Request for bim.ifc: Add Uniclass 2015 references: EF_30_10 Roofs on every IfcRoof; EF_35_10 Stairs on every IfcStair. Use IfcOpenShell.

First a look at what the model holds.

```python
import ifcopenshell

model = ifcopenshell.open("bim.ifc")
print(model.schema)
print("classifications:", [c.Name for c in model.by_type("IfcClassification")])
for ifc_class in ("IfcDoor", "IfcRoof", "IfcStair", "IfcWall", "IfcWindow"):
    print(ifc_class, len(model.by_type(ifc_class)))
```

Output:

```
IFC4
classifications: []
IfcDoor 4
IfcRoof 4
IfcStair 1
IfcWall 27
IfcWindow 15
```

```python
import ifcopenshell
import ifcopenshell.api.classification

model = ifcopenshell.open("bim.ifc")

system = ifcopenshell.api.classification.add_classification(model, classification="Uniclass 2015")

codes = {
    "IfcRoof": ("EF_30_10", "Roofs"),
    "IfcStair": ("EF_35_10", "Stairs"),
}
for ifc_class, (code, name) in codes.items():
    products = model.by_type(ifc_class)
    ifcopenshell.api.classification.add_reference(
        model, products=products, classification=system, identification=code, name=name
    )
    print(code, len(products))

model.write("bim-out.ifc")
```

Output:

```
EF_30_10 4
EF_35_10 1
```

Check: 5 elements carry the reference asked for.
